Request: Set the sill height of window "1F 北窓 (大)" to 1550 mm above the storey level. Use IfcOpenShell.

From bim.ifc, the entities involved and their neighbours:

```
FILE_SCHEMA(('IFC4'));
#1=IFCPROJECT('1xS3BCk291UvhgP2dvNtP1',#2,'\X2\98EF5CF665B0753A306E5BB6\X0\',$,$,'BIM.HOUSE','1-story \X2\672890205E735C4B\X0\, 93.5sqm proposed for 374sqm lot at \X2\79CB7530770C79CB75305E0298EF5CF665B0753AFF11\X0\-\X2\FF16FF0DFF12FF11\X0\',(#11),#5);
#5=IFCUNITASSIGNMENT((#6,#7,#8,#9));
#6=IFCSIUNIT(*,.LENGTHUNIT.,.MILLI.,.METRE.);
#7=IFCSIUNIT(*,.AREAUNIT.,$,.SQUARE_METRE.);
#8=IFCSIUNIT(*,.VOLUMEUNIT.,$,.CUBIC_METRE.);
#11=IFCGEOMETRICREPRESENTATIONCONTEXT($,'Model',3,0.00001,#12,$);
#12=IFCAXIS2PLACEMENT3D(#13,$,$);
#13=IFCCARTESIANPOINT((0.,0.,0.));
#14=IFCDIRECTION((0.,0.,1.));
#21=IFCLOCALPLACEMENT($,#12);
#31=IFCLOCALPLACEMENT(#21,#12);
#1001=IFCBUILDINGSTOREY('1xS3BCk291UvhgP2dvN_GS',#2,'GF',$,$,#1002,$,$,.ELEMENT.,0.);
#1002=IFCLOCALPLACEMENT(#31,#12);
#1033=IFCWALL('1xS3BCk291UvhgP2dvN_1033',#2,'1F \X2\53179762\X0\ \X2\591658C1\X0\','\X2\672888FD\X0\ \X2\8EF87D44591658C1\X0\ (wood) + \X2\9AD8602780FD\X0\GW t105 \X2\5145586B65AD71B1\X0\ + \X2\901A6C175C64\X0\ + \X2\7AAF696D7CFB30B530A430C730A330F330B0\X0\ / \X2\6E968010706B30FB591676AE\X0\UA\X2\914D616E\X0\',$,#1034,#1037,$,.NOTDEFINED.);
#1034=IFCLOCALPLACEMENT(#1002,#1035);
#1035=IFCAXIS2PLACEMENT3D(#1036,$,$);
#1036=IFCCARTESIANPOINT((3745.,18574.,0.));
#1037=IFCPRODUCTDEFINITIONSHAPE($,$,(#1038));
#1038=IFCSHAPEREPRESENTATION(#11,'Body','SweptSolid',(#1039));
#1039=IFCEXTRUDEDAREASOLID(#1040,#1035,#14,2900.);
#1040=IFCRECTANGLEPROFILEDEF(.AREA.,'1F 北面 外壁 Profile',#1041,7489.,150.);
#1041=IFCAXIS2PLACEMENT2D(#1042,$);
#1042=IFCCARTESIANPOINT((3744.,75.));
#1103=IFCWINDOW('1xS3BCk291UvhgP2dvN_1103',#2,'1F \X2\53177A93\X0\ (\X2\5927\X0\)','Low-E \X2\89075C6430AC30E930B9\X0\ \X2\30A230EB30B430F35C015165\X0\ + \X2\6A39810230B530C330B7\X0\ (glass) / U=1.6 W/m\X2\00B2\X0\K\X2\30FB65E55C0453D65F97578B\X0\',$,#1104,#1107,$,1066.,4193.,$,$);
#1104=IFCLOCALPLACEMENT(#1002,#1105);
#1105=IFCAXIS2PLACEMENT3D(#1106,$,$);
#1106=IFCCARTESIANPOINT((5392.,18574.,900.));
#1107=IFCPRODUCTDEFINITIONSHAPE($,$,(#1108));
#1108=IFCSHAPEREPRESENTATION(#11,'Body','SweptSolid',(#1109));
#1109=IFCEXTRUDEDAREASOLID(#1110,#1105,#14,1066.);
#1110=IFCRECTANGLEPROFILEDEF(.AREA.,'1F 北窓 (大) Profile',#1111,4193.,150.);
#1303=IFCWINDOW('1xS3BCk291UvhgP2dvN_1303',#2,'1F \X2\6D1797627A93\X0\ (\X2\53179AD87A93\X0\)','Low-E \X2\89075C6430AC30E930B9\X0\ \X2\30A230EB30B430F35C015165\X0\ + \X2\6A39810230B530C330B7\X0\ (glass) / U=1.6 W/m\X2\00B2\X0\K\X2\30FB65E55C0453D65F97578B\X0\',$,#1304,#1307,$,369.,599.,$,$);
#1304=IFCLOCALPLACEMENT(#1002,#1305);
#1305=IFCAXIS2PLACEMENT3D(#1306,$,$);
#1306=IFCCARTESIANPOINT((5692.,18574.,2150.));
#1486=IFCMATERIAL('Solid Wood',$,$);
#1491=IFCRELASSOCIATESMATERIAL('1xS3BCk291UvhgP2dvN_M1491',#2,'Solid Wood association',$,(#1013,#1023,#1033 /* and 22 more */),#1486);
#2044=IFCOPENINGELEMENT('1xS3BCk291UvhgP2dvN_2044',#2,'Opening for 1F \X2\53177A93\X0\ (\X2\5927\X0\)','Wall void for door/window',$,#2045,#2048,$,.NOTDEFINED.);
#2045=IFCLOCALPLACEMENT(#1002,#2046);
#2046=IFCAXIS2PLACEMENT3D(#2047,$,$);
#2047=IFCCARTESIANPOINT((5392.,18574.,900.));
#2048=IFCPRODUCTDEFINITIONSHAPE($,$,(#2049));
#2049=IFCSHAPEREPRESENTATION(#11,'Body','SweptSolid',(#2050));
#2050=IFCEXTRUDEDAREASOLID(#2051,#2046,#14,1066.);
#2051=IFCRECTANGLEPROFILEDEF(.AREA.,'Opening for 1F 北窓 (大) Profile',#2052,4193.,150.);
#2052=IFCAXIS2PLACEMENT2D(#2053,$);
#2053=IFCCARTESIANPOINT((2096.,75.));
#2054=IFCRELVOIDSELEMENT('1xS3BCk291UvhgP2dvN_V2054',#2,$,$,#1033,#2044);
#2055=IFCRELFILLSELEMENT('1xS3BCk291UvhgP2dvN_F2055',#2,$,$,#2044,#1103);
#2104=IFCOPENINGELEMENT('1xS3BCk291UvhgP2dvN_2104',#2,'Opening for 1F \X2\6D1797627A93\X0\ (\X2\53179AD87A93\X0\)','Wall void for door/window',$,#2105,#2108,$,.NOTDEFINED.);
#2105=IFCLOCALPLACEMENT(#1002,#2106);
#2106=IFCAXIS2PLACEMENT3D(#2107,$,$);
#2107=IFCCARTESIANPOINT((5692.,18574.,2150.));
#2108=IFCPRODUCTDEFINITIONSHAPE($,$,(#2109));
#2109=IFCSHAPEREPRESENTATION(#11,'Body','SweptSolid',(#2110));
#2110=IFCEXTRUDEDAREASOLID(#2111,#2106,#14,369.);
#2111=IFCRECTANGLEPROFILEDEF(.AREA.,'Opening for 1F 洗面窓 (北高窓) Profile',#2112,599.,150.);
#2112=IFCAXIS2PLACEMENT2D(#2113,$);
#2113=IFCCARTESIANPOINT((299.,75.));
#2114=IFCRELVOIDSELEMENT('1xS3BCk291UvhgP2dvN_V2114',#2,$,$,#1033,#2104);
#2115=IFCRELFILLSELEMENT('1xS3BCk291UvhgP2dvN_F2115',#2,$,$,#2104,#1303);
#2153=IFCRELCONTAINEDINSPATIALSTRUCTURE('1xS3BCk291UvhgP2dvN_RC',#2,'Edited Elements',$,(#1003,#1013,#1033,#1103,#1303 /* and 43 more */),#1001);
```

```python
import numpy as np
import ifcopenshell
import ifcopenshell.api.geometry
import ifcopenshell.geom
import ifcopenshell.util.element
import ifcopenshell.util.placement
import ifcopenshell.util.shape
import ifcopenshell.util.unit

model = ifcopenshell.open("bim.ifc")
unit_scale = ifcopenshell.util.unit.calculate_unit_scale(model)

window = model.by_guid("1xS3BCk291UvhgP2dvN_1103")
opening = window.FillsVoids[0].RelatingOpeningElement
storey = ifcopenshell.util.element.get_container(window, ifc_class="IfcBuildingStorey")
level = ifcopenshell.util.placement.get_local_placement(storey.ObjectPlacement)[2, 3]

# The opening's origin need not be at the sill, so measure its lowest point.
shape = ifcopenshell.geom.create_shape(ifcopenshell.geom.settings(), opening)
bottom = ifcopenshell.util.shape.get_shape_bottom_elevation(shape, shape.geometry) / unit_scale
dz = level + 1.55 / unit_scale - bottom

shift = np.array([0.0, 0.0, dz])
# The window is not placed relative to its opening, so move both.
for product in (opening, window):
    matrix = ifcopenshell.util.placement.get_local_placement(product.ObjectPlacement)
    matrix[:3, 3] += shift
    ifcopenshell.api.geometry.edit_object_placement(model, product=product, matrix=matrix, is_si=False)

print(f"moved by {dz * unit_scale:+.3f} m")

model.write("bim_rev.ifc")
```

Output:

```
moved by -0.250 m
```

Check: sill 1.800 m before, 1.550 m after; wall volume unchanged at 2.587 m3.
